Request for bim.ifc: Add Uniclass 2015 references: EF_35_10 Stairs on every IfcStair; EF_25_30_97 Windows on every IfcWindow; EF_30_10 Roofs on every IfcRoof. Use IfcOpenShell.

First a look at what the model holds.

```python
import ifcopenshell

model = ifcopenshell.open("bim.ifc")
print(model.schema)
print("classifications:", [c.Name for c in model.by_type("IfcClassification")])
for ifc_class in ("IfcDoor", "IfcRoof", "IfcStair", "IfcWall", "IfcWindow"):
    print(ifc_class, len(model.by_type(ifc_class)))
```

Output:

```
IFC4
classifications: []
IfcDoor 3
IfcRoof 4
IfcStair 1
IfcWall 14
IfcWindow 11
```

```python
import ifcopenshell
import ifcopenshell.api.classification

model = ifcopenshell.open("bim.ifc")

system = ifcopenshell.api.classification.add_classification(model, classification="Uniclass 2015")

codes = {
    "IfcStair": ("EF_35_10", "Stairs"),
    "IfcWindow": ("EF_25_30_97", "Windows"),
    "IfcRoof": ("EF_30_10", "Roofs"),
}
for ifc_class, (code, name) in codes.items():
    products = model.by_type(ifc_class)
    ifcopenshell.api.classification.add_reference(
        model, products=products, classification=system, identification=code, name=name
    )
    print(code, len(products))

model.write("bim_v2.ifc")
```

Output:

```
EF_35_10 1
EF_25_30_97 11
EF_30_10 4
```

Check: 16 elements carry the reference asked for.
